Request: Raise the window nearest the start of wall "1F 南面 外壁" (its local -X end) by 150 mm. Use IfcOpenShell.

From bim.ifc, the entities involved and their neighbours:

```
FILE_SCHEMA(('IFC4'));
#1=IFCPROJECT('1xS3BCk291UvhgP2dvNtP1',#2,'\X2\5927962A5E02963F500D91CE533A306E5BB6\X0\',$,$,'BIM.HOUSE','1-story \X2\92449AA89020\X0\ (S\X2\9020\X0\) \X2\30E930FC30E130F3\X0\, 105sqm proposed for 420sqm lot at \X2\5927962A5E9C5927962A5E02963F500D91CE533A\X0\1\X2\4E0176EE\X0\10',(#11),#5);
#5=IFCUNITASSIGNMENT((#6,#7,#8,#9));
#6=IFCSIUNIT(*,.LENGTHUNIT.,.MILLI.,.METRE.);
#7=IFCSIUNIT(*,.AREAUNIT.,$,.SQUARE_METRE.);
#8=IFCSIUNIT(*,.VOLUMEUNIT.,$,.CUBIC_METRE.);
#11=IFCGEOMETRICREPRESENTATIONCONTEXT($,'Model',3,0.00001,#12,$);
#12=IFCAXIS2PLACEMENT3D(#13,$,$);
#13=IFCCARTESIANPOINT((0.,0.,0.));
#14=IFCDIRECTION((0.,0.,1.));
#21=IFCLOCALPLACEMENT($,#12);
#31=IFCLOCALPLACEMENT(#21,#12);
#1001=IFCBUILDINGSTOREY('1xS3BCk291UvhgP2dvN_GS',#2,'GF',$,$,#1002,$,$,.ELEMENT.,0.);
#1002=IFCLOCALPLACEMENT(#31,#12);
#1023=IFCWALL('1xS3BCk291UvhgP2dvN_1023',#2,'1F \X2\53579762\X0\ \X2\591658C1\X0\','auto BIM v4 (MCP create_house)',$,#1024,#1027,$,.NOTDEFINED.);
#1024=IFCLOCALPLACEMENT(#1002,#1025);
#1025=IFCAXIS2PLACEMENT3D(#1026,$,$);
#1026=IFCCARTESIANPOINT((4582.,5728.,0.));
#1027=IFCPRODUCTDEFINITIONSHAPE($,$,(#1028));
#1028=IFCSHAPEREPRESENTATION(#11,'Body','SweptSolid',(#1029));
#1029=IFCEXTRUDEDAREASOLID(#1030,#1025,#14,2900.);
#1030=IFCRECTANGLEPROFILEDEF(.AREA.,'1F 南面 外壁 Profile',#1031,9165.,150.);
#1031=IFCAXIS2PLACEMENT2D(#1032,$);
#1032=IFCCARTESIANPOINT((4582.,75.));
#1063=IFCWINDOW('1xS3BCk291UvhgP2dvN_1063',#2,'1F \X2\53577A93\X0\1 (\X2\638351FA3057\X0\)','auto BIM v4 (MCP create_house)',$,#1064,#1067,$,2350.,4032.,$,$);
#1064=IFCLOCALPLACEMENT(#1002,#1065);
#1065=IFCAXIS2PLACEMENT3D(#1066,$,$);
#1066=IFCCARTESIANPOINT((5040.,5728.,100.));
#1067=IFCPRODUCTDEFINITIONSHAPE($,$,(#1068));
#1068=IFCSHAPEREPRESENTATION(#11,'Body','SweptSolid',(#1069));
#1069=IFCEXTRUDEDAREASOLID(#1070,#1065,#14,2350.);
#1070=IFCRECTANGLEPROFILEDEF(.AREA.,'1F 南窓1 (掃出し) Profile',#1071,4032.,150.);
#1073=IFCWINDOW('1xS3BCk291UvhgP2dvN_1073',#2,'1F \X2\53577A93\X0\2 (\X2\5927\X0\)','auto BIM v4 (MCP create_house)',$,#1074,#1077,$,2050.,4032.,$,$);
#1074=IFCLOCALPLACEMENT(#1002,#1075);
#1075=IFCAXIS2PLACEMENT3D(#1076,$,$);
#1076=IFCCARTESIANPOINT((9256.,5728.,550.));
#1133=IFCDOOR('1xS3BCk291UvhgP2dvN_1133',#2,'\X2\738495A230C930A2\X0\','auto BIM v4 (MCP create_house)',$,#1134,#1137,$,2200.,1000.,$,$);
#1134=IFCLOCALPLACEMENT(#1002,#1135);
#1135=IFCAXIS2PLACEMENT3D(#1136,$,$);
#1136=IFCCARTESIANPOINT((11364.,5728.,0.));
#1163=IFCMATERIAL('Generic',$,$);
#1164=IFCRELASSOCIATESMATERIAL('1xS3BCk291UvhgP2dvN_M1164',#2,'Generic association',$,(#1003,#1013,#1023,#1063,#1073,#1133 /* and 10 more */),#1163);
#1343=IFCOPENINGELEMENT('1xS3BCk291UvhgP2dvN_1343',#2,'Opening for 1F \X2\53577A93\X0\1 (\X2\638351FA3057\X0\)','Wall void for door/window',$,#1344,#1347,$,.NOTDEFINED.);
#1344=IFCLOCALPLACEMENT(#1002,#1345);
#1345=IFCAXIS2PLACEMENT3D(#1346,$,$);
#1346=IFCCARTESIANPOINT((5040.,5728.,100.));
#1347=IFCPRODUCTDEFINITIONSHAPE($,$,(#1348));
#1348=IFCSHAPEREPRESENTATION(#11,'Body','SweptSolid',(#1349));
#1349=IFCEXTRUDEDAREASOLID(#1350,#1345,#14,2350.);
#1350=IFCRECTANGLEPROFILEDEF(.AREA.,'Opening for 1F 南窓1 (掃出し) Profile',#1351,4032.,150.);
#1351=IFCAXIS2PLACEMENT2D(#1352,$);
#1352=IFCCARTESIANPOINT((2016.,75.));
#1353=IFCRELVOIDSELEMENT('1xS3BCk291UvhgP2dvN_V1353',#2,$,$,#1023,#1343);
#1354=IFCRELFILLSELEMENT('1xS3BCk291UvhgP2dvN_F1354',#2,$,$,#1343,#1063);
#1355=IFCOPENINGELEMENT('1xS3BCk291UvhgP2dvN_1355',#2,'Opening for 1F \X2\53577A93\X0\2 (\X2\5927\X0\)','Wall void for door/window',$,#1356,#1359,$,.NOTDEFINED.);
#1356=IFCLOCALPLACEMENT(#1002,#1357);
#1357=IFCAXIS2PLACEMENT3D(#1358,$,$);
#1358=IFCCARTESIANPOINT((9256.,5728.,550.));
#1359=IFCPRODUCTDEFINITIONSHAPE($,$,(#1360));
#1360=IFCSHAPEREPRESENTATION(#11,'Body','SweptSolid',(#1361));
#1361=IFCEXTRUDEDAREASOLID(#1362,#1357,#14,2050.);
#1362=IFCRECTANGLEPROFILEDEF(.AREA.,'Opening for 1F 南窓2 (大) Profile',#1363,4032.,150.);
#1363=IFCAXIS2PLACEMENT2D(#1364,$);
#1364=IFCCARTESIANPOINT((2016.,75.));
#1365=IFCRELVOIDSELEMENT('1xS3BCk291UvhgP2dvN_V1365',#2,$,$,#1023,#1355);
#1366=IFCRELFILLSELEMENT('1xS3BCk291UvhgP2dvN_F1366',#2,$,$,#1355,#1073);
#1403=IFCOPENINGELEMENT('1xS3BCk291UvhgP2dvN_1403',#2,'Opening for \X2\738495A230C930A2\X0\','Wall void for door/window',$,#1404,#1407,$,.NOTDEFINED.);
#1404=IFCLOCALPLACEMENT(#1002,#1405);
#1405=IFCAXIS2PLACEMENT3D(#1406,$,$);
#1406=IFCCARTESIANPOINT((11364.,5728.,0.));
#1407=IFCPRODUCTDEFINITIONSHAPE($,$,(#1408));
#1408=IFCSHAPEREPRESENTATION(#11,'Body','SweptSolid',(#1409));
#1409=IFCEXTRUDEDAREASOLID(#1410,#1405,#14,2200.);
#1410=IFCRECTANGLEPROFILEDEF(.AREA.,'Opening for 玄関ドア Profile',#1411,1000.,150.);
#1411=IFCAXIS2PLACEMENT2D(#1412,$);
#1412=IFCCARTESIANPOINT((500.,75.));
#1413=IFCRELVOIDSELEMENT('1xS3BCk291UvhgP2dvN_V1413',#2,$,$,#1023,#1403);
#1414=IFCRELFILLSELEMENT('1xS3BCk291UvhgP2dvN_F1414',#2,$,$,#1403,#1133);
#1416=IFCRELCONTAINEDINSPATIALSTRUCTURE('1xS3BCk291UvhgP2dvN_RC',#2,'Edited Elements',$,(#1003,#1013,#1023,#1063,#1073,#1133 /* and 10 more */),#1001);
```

```python
import numpy as np
import ifcopenshell
import ifcopenshell.api.geometry
import ifcopenshell.util.placement
import ifcopenshell.util.unit

model = ifcopenshell.open("bim.ifc")
unit_scale = ifcopenshell.util.unit.calculate_unit_scale(model)

window = model.by_guid("1xS3BCk291UvhgP2dvN_1063")
opening = window.FillsVoids[0].RelatingOpeningElement
dz = 150.0

shift = np.array([0.0, 0.0, dz])
# The window is not placed relative to its opening, so move both.
for product in (opening, window):
    matrix = ifcopenshell.util.placement.get_local_placement(product.ObjectPlacement)
    matrix[:3, 3] += shift
    ifcopenshell.api.geometry.edit_object_placement(model, product=product, matrix=matrix, is_si=False)

print(f"moved by {dz * unit_scale:+.3f} m")

model.write("bim_updated.ifc")
```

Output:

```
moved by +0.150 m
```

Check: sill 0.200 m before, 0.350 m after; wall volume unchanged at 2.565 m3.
